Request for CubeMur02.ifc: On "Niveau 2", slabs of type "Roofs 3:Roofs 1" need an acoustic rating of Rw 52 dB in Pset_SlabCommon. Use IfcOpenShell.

First a look at what the model holds.

```python
import ifcopenshell
import ifcopenshell.util.element

model = ifcopenshell.open("CubeMur02.ifc")
print(model.schema)
storey = next(s for s in model.by_type("IfcBuildingStorey") if s.Name == "Niveau 2")
slabs = [e for e in ifcopenshell.util.element.get_decomposition(storey) if e.is_a("IfcSlab")]
seen = {}
for e in slabs:
    element_type = ifcopenshell.util.element.get_type(e)
    key = (element_type.Name if element_type != e and element_type else None, ifcopenshell.util.element.get_pset(e, "Pset_SlabCommon", "AcousticRating"))
    seen[key] = seen.get(key, 0) + 1
for (name, value), count in sorted(seen.items(), key=str):
    print(count, "x", name, "|", value)
```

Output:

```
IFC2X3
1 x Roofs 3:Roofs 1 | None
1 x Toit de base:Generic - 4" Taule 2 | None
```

```python
import ifcopenshell
import ifcopenshell.api.pset
import ifcopenshell.util.element

model = ifcopenshell.open("CubeMur02.ifc")

storey = next(s for s in model.by_type("IfcBuildingStorey") if s.Name == "Niveau 2")
slabs = [e for e in ifcopenshell.util.element.get_decomposition(storey) if e.is_a("IfcSlab")]

count = 0
for e in slabs:
    element_type = ifcopenshell.util.element.get_type(e)
    if element_type in (None, e) or element_type.Name != "Roofs 3:Roofs 1":
        continue
    # add_pset returns the element's existing set when there is one.
    pset = ifcopenshell.api.pset.add_pset(model, product=e, name="Pset_SlabCommon")
    ifcopenshell.api.pset.edit_pset(model, pset=pset, properties={"AcousticRating": "Rw 52 dB"})
    count += 1

print(count, "slabs updated")

model.write("CubeMur02_rev.ifc")
```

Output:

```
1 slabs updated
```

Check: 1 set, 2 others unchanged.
